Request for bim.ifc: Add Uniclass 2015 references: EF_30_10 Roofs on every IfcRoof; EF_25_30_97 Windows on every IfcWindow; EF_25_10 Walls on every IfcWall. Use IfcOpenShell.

First a look at what the model holds.

```python
import ifcopenshell

model = ifcopenshell.open("bim.ifc")
print(model.schema)
print("classifications:", [c.Name for c in model.by_type("IfcClassification")])
for ifc_class in ("IfcDoor", "IfcRoof", "IfcStair", "IfcWall", "IfcWindow"):
    print(ifc_class, len(model.by_type(ifc_class)))
```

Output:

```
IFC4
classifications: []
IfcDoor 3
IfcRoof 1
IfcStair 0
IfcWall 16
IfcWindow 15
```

```python
import ifcopenshell
import ifcopenshell.api.classification

model = ifcopenshell.open("bim.ifc")

system = ifcopenshell.api.classification.add_classification(model, classification="Uniclass 2015")

codes = {
    "IfcRoof": ("EF_30_10", "Roofs"),
    "IfcWindow": ("EF_25_30_97", "Windows"),
    "IfcWall": ("EF_25_10", "Walls"),
}
for ifc_class, (code, name) in codes.items():
    products = model.by_type(ifc_class)
    ifcopenshell.api.classification.add_reference(
        model, products=products, classification=system, identification=code, name=name
    )
    print(code, len(products))

model.write("bim_v2.ifc")
```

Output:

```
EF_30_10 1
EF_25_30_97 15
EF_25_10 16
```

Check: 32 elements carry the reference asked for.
